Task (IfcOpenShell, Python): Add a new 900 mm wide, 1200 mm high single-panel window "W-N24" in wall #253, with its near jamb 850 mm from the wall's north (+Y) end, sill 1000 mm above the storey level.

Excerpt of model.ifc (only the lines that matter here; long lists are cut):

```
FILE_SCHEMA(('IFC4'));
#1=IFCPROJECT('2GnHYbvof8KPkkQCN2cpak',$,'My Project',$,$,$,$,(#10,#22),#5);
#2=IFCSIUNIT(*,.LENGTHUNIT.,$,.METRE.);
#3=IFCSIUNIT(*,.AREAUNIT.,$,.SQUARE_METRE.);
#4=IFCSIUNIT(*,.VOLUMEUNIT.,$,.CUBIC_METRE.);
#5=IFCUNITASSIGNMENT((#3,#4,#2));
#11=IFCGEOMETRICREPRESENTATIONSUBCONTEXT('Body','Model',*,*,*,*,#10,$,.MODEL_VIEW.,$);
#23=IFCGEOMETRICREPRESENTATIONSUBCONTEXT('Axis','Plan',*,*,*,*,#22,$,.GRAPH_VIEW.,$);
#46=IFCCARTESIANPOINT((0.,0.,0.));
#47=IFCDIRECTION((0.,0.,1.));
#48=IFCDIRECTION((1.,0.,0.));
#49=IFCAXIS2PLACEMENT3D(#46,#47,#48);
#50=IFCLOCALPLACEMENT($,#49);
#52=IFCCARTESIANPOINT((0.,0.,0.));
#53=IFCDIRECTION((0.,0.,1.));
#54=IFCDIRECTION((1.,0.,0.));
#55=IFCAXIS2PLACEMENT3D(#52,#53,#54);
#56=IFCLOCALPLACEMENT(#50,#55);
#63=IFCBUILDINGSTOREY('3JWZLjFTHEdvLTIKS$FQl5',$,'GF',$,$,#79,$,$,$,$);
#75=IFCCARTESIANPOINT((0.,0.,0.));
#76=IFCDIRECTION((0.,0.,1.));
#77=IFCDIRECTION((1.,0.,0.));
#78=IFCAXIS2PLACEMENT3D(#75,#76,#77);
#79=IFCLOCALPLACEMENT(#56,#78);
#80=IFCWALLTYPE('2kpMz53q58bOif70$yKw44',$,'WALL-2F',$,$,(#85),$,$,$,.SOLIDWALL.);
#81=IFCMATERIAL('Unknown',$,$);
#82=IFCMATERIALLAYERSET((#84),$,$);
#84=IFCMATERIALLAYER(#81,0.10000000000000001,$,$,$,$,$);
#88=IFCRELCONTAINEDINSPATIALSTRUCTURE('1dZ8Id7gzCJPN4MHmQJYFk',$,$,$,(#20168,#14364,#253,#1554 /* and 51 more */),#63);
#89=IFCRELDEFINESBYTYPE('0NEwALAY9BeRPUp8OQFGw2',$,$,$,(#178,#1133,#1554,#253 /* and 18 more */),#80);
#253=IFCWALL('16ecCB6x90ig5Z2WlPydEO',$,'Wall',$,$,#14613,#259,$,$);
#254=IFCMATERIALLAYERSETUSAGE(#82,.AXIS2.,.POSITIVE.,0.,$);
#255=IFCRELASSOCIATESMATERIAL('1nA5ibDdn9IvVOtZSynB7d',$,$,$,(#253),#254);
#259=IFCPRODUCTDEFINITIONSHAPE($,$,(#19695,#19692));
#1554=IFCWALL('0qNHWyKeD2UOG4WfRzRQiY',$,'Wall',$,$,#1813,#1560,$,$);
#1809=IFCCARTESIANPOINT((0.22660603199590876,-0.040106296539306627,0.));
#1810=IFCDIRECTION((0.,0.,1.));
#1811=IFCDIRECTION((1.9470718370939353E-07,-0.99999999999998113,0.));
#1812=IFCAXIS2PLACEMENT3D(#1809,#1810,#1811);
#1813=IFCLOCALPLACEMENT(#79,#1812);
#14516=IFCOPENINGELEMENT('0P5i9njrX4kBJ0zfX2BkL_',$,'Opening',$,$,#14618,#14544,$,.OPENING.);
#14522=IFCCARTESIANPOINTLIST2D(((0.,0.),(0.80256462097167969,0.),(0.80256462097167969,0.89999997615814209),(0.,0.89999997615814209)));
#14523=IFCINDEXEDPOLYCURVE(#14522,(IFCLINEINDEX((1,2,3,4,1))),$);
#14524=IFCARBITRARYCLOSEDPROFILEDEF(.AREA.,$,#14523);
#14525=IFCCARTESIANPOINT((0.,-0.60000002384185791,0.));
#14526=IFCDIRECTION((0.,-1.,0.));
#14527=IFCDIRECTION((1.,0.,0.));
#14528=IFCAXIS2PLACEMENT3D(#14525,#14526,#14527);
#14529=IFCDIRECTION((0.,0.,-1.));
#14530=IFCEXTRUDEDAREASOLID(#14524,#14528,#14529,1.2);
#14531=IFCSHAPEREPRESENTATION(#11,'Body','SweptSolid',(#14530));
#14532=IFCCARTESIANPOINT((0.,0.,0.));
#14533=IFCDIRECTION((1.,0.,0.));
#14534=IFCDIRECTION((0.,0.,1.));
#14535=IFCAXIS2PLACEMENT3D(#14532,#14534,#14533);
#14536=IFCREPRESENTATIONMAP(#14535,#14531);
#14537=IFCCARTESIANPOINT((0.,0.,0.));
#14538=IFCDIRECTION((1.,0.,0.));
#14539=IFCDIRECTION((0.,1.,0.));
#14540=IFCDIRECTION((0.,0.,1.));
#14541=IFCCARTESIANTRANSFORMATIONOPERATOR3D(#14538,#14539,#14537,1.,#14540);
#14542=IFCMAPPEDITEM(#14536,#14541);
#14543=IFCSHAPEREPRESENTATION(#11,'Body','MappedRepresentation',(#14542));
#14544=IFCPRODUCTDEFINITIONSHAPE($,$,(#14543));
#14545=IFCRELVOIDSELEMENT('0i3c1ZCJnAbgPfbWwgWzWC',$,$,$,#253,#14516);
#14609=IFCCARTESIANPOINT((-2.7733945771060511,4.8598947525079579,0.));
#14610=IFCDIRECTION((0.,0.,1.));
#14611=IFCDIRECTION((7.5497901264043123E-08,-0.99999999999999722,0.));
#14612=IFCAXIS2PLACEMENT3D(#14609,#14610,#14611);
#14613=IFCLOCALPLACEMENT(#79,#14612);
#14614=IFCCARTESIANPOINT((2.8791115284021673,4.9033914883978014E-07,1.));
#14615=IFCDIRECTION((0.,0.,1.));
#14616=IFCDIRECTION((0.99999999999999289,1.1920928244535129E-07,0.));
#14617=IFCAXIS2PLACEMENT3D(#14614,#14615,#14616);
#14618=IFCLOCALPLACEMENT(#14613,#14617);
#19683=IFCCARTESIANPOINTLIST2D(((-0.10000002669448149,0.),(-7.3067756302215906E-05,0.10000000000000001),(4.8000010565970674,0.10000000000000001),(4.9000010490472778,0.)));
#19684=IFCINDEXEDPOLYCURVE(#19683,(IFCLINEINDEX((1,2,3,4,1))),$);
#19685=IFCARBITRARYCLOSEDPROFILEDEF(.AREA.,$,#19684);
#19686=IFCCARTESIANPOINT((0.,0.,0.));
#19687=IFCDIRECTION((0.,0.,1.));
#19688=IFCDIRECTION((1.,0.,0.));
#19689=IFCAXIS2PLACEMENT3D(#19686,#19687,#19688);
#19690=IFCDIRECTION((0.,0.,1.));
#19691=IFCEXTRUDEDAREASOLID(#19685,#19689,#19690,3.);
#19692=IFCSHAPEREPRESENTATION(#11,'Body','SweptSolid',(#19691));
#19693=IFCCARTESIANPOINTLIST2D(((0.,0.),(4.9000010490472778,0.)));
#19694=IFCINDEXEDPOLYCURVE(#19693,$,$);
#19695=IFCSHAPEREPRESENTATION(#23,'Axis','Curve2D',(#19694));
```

```python
import numpy as np
import ifcopenshell
import ifcopenshell.api.feature
import ifcopenshell.api.geometry
import ifcopenshell.api.root
import ifcopenshell.api.spatial
import ifcopenshell.geom
import ifcopenshell.util.element
import ifcopenshell.util.placement
import ifcopenshell.util.representation
import ifcopenshell.util.shape
import ifcopenshell.util.unit

model = ifcopenshell.open("model.ifc")
unit_scale = ifcopenshell.util.unit.calculate_unit_scale(model)
settings = ifcopenshell.geom.settings()


def volume(element):
    """Net volume in cubic metres, openings subtracted."""
    shape = ifcopenshell.geom.create_shape(settings, element)
    return ifcopenshell.util.shape.get_volume(shape.geometry)


wall = model.by_guid("16ecCB6x90ig5Z2WlPydEO")
storey = ifcopenshell.util.element.get_container(wall, ifc_class="IfcBuildingStorey")
context = ifcopenshell.util.representation.get_context(model, "Model", "Body", "MODEL_VIEW")
before = volume(wall)

width, height, from_end, sill = 0.9, 1.2, 0.85, 1  # metres

# The wall runs along its own X axis, and the end named is its -X end.
wall_shape = ifcopenshell.geom.create_shape(settings, wall)
x, y, z = ifcopenshell.util.shape.get_vertices(wall_shape.geometry).T
start = x.min() + from_end
face, thickness = float(y.min()), float(y.max() - y.min())
wall_matrix = ifcopenshell.util.placement.get_local_placement(wall.ObjectPlacement)
level = ifcopenshell.util.placement.get_local_placement(storey.ObjectPlacement)[2, 3]


def in_wall(x, y):
    """Placement at x, y metres in the wall's axes, at sill height."""
    matrix = wall_matrix.copy()
    matrix[:, 3] = wall_matrix @ np.array([x / unit_scale, y / unit_scale, 0.0, 1.0])
    matrix[2, 3] = level + sill / unit_scale
    return matrix


# Opening: a box that overshoots both wall faces by 50 mm.
opening = ifcopenshell.api.root.create_entity(model, ifc_class="IfcOpeningElement", predefined_type="OPENING")
box = ifcopenshell.api.geometry.add_wall_representation(
    model, context=context, length=width, height=height, thickness=thickness + 0.1
)
ifcopenshell.api.geometry.assign_representation(model, product=opening, representation=box)
ifcopenshell.api.geometry.edit_object_placement(model, product=opening, matrix=in_wall(start, face - 0.05), is_si=False)
ifcopenshell.api.feature.add_feature(model, feature=opening, element=wall)

window = ifcopenshell.api.root.create_entity(model, ifc_class="IfcWindow", name="W-N24", predefined_type="WINDOW")
window.OverallWidth, window.OverallHeight = width / unit_scale, height / unit_scale
window.PartitioningType = "SINGLE_PANEL"
body = ifcopenshell.api.geometry.add_window_representation(
    model,
    context=context,
    overall_width=window.OverallWidth,
    overall_height=window.OverallHeight,
    partition_type="SINGLE_PANEL",
)
ifcopenshell.api.geometry.assign_representation(model, product=window, representation=body)
ifcopenshell.api.spatial.assign_container(model, products=[window], relating_structure=storey)
ifcopenshell.api.feature.add_filling(model, opening=opening, element=window)

# Centre the window in the wall's thickness.
ifcopenshell.api.geometry.edit_object_placement(model, product=window, matrix=in_wall(start, face), is_si=False)
window_shape = ifcopenshell.geom.create_shape(settings, window)
depth = ifcopenshell.util.shape.get_vertices(window_shape.geometry)[:, 1]
offset = face + thickness / 2 - (depth.min() + depth.max()) / 2
ifcopenshell.api.geometry.edit_object_placement(model, product=window, matrix=in_wall(start, offset), is_si=False)

after = volume(wall)

print(f"wall volume {before:.3f} -> {after:.3f} m3")

model.write("model_updated.ifc")
```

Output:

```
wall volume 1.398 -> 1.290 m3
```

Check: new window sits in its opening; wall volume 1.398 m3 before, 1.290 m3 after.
